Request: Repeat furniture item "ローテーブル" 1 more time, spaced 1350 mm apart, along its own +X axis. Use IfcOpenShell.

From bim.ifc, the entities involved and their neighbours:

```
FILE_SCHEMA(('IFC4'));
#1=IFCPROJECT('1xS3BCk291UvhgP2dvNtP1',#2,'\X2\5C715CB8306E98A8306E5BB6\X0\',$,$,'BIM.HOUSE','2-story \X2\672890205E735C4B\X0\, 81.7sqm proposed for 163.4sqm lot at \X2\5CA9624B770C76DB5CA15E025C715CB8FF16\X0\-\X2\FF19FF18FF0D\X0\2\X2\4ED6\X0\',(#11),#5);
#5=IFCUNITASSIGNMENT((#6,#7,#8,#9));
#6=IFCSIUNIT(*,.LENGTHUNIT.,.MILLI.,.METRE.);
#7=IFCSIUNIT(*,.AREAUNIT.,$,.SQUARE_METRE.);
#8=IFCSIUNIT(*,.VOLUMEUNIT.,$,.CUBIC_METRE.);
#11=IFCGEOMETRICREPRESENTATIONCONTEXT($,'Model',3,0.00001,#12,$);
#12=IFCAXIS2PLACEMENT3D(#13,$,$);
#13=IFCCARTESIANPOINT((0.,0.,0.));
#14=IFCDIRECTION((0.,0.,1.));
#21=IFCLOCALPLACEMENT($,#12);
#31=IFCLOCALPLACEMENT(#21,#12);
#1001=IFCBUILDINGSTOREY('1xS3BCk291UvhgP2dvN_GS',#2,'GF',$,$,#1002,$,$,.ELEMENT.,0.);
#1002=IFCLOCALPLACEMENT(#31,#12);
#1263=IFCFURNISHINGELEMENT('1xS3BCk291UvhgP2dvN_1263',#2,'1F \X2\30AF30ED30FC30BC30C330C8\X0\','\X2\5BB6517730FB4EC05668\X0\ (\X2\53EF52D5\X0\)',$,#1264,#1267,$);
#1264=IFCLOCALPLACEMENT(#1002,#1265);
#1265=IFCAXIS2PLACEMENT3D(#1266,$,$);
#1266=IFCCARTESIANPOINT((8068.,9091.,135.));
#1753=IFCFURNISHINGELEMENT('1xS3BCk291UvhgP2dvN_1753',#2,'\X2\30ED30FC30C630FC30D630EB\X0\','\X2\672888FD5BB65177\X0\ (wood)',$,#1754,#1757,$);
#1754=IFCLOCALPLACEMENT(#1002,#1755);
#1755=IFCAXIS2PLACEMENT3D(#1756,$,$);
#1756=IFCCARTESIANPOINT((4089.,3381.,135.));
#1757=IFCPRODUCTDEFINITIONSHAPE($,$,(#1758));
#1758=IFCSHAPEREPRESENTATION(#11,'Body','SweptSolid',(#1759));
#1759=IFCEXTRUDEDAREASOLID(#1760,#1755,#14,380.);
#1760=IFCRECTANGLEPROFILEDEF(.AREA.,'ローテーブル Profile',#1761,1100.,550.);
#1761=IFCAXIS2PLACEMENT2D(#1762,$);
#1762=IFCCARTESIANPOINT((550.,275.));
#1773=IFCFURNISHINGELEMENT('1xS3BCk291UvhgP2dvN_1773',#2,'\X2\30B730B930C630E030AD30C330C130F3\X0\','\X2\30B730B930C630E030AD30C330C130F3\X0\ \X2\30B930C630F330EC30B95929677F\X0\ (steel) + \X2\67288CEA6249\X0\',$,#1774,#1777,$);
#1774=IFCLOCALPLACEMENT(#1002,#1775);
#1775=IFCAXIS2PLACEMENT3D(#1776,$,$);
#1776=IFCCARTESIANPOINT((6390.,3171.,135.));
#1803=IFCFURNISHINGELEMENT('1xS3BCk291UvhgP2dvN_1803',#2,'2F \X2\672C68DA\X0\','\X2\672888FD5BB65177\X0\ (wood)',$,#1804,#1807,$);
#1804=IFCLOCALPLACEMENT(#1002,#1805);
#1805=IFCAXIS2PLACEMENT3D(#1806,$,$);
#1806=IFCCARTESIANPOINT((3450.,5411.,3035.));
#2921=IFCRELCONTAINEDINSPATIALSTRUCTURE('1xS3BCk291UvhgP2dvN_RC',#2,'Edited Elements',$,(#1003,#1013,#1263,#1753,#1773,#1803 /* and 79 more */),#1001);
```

```python
import ifcopenshell
import ifcopenshell.api.geometry
import ifcopenshell.api.root
import ifcopenshell.util.element
import ifcopenshell.util.placement
import ifcopenshell.util.unit

model = ifcopenshell.open("bim.ifc")
unit_scale = ifcopenshell.util.unit.calculate_unit_scale(model)


def reuse_history(source, copy):
    """copy_class also copies each property set's owner history, people and application; keep the originals."""
    for rel in copy.IsDefinedBy:
        if rel.is_a("IfcRelDefinesByProperties") and (history := rel.RelatingPropertyDefinition.OwnerHistory):
            rel.RelatingPropertyDefinition.OwnerHistory = source.OwnerHistory
            ifcopenshell.util.element.remove_deep2(model, history)


source = model.by_guid("1xS3BCk291UvhgP2dvN_1753")
base = ifcopenshell.util.placement.get_local_placement(source.ObjectPlacement)
step = base[:3, 0] * 1.35 / unit_scale

for i in range(1, 2):
    copy = ifcopenshell.api.root.copy_class(model, product=source)
    copy.Representation = ifcopenshell.util.element.copy_deep(
        model, source.Representation, exclude=["IfcGeometricRepresentationContext", "IfcRepresentationMap"]
    )
    reuse_history(source, copy)
    matrix = base.copy()
    matrix[:3, 3] += i * step
    print("added at", matrix[:3, 3].round(3) + 0.0)
    ifcopenshell.api.geometry.edit_object_placement(model, product=copy, matrix=matrix, is_si=False)

model.write("bim_updated.ifc")
```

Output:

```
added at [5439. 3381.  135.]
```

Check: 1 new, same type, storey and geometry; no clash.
